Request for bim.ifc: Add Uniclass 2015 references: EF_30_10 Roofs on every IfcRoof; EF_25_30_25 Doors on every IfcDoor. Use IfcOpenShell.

First a look at what the model holds.

```python
import ifcopenshell

model = ifcopenshell.open("bim.ifc")
print(model.schema)
print("classifications:", [c.Name for c in model.by_type("IfcClassification")])
for ifc_class in ("IfcDoor", "IfcRoof", "IfcStair", "IfcWall", "IfcWindow"):
    print(ifc_class, len(model.by_type(ifc_class)))
```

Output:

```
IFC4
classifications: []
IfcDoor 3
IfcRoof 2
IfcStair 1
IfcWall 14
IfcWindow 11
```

```python
import ifcopenshell
import ifcopenshell.api.classification

model = ifcopenshell.open("bim.ifc")

system = ifcopenshell.api.classification.add_classification(model, classification="Uniclass 2015")

codes = {
    "IfcRoof": ("EF_30_10", "Roofs"),
    "IfcDoor": ("EF_25_30_25", "Doors"),
}
for ifc_class, (code, name) in codes.items():
    products = model.by_type(ifc_class)
    ifcopenshell.api.classification.add_reference(
        model, products=products, classification=system, identification=code, name=name
    )
    print(code, len(products))

model.write("bim_updated.ifc")
```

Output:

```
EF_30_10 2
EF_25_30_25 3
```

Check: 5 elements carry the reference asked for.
